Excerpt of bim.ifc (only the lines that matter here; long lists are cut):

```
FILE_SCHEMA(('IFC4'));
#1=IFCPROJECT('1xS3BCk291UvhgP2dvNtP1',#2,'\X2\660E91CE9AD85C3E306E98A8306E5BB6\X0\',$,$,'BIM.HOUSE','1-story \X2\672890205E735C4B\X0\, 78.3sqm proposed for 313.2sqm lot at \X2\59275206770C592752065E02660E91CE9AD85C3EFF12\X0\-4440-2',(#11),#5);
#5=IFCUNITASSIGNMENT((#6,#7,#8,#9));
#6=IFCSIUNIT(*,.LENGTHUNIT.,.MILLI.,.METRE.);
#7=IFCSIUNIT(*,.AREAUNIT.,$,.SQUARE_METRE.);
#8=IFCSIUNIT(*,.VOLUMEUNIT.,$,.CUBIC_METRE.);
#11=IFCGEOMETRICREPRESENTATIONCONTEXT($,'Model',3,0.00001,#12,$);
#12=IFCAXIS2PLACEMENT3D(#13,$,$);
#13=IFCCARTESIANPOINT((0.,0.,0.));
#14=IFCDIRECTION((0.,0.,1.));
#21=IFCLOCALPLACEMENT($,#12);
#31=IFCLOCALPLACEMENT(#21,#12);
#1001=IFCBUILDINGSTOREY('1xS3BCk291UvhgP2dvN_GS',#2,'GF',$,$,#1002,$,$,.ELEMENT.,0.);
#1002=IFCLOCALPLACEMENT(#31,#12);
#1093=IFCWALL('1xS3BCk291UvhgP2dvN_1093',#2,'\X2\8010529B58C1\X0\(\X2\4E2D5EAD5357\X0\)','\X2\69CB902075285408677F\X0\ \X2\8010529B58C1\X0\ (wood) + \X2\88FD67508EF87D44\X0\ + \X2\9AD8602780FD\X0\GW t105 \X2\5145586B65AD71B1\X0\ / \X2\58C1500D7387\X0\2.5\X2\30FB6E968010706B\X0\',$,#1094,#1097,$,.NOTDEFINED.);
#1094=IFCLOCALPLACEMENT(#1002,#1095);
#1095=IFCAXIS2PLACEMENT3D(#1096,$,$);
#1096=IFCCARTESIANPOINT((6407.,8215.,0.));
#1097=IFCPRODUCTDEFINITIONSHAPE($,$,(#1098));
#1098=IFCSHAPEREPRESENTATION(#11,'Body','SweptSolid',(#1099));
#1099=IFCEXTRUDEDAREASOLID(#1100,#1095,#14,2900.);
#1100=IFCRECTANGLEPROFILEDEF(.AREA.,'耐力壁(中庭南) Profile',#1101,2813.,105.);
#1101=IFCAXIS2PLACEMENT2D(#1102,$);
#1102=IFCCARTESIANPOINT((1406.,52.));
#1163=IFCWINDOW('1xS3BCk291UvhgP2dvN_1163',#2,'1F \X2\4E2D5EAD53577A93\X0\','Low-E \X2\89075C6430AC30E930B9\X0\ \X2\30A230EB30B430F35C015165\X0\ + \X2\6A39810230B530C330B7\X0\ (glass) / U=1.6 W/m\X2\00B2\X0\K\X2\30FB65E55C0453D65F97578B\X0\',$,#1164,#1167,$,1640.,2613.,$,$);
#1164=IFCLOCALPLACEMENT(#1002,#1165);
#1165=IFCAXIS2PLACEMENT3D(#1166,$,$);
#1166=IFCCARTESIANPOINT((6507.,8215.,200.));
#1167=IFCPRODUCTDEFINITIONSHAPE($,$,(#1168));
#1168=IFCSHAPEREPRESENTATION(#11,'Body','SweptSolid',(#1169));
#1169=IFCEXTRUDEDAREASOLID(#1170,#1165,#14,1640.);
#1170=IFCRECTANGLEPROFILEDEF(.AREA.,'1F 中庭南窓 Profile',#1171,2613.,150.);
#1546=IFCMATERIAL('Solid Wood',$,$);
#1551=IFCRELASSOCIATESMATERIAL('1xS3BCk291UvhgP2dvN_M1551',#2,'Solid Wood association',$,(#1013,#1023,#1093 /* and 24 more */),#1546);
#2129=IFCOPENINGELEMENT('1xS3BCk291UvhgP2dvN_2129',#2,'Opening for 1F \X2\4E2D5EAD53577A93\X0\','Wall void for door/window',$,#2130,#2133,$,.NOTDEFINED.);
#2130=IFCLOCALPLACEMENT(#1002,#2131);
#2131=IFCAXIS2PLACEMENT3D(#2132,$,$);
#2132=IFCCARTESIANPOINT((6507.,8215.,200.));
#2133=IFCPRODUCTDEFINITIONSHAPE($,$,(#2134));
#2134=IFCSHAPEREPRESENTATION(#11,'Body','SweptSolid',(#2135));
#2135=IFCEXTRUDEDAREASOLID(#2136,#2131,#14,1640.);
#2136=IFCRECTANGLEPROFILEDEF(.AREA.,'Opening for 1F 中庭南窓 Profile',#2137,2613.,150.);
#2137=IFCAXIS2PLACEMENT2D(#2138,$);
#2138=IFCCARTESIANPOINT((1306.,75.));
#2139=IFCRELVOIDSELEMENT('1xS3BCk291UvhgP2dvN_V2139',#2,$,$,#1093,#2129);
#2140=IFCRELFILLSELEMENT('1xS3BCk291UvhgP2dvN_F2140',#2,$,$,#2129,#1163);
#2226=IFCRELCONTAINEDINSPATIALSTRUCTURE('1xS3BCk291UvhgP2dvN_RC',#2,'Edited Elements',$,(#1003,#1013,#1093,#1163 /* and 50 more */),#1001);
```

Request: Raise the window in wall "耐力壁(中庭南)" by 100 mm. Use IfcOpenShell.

```python
import numpy as np
import ifcopenshell
import ifcopenshell.api.geometry
import ifcopenshell.util.placement
import ifcopenshell.util.unit

model = ifcopenshell.open("bim.ifc")
unit_scale = ifcopenshell.util.unit.calculate_unit_scale(model)

window = model.by_guid("1xS3BCk291UvhgP2dvN_1163")
opening = window.FillsVoids[0].RelatingOpeningElement
dz = 0.1 / unit_scale

shift = np.array([0.0, 0.0, dz])
# The window is not placed relative to its opening, so move both.
for product in (opening, window):
    matrix = ifcopenshell.util.placement.get_local_placement(product.ObjectPlacement)
    matrix[:3, 3] += shift
    ifcopenshell.api.geometry.edit_object_placement(model, product=product, matrix=matrix, is_si=False)

print(f"moved by {dz * unit_scale:+.3f} m")

model.write("bim_rev.ifc")
```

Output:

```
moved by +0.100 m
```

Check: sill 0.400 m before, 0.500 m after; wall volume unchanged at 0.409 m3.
